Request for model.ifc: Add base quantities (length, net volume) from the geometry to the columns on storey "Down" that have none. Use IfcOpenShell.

First a look at what the model holds.

```python
import ifcopenshell
import ifcopenshell.util.element
import ifcopenshell.util.unit

model = ifcopenshell.open("model.ifc")
print(model.schema)
for unit_type in ("LENGTHUNIT", "AREAUNIT", "VOLUMEUNIT"):
    print(unit_type, ifcopenshell.util.unit.calculate_unit_scale(model, unit_type))
storey = next(s for s in model.by_type("IfcBuildingStorey") if s.Name == "Down")
columns = [e for e in ifcopenshell.util.element.get_decomposition(storey) if e.is_a("IfcColumn")]
for e in sorted(columns, key=lambda e: e.id()):
    print(e.id(), e.is_a(), e.Name, list(ifcopenshell.util.element.get_psets(e, qtos_only=True)), sep=" | ")
```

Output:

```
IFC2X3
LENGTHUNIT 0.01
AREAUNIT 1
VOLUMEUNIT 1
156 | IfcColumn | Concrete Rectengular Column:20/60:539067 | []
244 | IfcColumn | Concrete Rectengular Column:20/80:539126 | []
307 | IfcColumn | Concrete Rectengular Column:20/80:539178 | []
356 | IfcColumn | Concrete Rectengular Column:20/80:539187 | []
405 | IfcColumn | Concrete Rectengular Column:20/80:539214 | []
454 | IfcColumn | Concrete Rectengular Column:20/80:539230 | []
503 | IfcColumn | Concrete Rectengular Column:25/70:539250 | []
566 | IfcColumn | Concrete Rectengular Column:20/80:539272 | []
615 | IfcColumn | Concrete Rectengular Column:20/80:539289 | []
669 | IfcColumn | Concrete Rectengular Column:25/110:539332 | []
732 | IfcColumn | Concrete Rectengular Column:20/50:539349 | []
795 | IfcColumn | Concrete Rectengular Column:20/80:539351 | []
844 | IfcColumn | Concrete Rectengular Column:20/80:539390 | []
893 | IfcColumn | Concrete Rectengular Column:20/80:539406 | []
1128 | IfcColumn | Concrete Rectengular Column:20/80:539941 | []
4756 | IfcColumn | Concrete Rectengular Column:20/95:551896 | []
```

```python
import ifcopenshell
import ifcopenshell.api.pset
import ifcopenshell.geom
import ifcopenshell.util.element
import ifcopenshell.util.shape
import ifcopenshell.util.unit

model = ifcopenshell.open("model.ifc")
unit_scale = ifcopenshell.util.unit.calculate_unit_scale(model)
volume_scale = ifcopenshell.util.unit.calculate_unit_scale(model, "VOLUMEUNIT")
settings = ifcopenshell.geom.settings()

storey = next(s for s in model.by_type("IfcBuildingStorey") if s.Name == "Down")
columns = [e for e in ifcopenshell.util.element.get_decomposition(storey) if e.is_a("IfcColumn")]

for e in sorted(columns, key=lambda e: e.id()):
    if ifcopenshell.util.element.get_psets(e, qtos_only=True, should_inherit=False):
        continue
    # Geometry comes back in metres, in the element's own axes.
    shape = ifcopenshell.geom.create_shape(settings, e)
    values = {
        "Length": ifcopenshell.util.shape.get_z(shape.geometry) / unit_scale,
        "NetVolume": ifcopenshell.util.shape.get_volume(shape.geometry) / volume_scale,
    }
    qto = ifcopenshell.api.pset.add_qto(model, product=e, name="BaseQuantities")
    ifcopenshell.api.pset.edit_qto(model, qto=qto, properties=values)
    print(e.id(), {k: round(v, 3) for k, v in values.items()})

model.write("model_edited.ifc")
```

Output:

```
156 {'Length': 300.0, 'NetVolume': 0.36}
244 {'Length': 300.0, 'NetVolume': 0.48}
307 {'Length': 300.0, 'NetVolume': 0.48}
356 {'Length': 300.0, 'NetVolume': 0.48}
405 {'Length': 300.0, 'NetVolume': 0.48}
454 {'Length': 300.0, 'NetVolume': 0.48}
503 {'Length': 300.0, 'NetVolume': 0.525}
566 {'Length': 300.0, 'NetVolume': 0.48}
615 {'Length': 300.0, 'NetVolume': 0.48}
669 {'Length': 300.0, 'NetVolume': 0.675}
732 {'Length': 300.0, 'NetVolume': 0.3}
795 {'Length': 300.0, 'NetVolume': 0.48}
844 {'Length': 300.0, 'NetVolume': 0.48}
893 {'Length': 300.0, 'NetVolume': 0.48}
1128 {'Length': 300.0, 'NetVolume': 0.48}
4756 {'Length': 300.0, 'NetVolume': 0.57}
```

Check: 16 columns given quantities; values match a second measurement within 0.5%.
